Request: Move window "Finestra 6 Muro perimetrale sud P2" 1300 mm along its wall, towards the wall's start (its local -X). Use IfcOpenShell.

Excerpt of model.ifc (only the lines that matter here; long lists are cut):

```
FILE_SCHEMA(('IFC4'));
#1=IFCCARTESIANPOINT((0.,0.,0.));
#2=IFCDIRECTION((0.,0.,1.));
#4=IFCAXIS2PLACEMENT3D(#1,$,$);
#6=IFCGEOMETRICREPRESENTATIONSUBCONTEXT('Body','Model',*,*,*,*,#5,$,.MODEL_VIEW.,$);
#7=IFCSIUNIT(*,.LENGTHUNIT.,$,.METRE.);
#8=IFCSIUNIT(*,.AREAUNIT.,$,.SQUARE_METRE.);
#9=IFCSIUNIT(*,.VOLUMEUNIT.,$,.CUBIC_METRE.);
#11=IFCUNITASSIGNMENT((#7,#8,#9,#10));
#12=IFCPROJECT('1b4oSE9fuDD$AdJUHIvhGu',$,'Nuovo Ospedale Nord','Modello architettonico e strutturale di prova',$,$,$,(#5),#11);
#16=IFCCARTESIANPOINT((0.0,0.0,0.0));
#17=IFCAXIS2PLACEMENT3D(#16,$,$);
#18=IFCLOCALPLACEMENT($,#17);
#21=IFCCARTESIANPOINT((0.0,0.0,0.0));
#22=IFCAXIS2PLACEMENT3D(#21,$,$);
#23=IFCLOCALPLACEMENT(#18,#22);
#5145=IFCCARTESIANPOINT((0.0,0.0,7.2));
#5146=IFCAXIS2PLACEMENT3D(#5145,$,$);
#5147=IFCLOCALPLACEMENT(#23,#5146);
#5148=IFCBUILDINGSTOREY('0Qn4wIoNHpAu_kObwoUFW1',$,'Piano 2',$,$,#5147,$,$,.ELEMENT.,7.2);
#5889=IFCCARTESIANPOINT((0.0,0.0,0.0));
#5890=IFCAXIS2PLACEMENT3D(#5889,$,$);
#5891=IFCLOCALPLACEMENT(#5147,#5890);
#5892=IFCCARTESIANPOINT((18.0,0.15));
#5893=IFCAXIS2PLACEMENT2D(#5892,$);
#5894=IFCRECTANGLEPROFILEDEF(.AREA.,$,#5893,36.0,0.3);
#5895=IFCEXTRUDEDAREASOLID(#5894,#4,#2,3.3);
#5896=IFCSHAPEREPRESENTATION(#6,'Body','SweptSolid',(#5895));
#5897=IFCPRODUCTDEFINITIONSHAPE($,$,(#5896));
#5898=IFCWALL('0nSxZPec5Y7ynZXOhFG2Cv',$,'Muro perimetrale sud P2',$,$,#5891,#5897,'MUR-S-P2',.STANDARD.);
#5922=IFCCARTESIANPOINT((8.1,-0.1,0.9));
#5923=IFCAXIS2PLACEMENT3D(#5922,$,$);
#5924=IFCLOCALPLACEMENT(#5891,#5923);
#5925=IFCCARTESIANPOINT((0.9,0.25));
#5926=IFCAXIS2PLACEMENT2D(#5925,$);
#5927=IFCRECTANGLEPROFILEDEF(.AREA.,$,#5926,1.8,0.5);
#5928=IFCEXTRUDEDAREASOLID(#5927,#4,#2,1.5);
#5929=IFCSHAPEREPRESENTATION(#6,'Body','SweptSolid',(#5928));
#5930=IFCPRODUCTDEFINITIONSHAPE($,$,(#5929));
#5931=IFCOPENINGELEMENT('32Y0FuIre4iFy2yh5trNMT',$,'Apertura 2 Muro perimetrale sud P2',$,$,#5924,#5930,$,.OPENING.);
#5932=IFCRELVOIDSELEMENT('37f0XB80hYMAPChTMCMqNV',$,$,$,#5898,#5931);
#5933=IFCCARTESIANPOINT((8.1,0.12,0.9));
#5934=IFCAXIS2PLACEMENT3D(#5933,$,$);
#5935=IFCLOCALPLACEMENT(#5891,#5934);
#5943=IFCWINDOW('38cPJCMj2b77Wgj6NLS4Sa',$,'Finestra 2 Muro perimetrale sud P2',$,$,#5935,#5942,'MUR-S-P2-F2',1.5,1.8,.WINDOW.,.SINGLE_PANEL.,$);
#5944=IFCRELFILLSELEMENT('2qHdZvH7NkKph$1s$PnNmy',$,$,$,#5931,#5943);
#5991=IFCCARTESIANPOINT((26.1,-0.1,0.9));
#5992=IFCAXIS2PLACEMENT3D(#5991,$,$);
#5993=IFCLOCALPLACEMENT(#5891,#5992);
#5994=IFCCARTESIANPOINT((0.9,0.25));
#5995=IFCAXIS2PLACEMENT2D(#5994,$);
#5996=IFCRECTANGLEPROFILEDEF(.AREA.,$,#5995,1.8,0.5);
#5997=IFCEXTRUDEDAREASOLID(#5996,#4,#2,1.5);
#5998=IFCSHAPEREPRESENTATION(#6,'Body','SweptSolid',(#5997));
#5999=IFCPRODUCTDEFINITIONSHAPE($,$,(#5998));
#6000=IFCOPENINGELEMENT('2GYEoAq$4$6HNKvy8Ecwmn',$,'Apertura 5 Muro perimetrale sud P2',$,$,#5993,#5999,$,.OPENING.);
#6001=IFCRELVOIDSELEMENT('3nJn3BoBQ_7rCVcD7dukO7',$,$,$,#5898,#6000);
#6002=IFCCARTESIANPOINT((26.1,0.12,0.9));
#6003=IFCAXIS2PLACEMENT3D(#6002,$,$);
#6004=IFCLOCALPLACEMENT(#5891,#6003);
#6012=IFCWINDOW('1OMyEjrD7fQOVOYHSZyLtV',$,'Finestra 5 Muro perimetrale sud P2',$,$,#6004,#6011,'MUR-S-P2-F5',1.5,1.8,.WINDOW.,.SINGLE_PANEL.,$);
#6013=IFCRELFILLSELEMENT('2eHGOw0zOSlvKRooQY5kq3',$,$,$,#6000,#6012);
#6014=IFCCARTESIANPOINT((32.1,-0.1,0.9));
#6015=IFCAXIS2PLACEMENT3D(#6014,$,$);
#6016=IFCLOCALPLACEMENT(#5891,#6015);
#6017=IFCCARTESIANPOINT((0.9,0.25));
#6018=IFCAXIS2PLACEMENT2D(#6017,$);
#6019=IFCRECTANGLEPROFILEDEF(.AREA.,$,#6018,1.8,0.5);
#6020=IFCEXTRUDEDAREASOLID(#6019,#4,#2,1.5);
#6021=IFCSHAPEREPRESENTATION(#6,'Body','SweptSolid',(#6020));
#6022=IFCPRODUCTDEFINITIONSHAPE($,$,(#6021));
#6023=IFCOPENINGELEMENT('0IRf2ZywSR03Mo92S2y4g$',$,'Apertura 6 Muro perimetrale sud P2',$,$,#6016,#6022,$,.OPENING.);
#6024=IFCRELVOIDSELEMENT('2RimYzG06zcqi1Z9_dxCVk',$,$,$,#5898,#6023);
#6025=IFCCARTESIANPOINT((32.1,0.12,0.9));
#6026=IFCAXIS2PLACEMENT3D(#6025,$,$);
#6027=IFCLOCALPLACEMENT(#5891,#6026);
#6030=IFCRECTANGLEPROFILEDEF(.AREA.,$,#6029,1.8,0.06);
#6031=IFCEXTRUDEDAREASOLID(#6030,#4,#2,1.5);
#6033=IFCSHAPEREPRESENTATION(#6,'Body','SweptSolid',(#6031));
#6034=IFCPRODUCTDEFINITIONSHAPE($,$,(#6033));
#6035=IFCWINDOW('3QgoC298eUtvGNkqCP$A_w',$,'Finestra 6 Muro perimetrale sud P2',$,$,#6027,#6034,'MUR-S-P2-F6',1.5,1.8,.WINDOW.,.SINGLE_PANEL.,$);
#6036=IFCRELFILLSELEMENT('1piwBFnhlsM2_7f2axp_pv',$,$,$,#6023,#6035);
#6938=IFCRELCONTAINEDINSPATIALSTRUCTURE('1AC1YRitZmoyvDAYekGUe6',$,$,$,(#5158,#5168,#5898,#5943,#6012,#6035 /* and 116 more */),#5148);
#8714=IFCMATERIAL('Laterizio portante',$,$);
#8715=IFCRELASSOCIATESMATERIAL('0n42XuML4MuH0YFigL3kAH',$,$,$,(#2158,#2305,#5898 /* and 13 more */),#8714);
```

```python
import ifcopenshell
import ifcopenshell.api.geometry
import ifcopenshell.util.placement
import ifcopenshell.util.unit

model = ifcopenshell.open("model.ifc")
unit_scale = ifcopenshell.util.unit.calculate_unit_scale(model)

window = model.by_guid("3QgoC298eUtvGNkqCP$A_w")
opening = window.FillsVoids[0].RelatingOpeningElement
wall = opening.VoidsElements[0].RelatingBuildingElement

wall_matrix = ifcopenshell.util.placement.get_local_placement(wall.ObjectPlacement)
shift = wall_matrix[:3, 0] * -1.3 / unit_scale
before = ifcopenshell.util.placement.get_local_placement(window.ObjectPlacement)[:3, 3].copy()

# The window is not placed relative to its opening, so move both.
for product in (opening, window):
    matrix = ifcopenshell.util.placement.get_local_placement(product.ObjectPlacement)
    matrix[:3, 3] += shift
    ifcopenshell.api.geometry.edit_object_placement(model, product=product, matrix=matrix, is_si=False)

after = ifcopenshell.util.placement.get_local_placement(window.ObjectPlacement)[:3, 3]
print("window moved by", (after - before).round(3) + 0.0)

model.write("model_edited.ifc")
```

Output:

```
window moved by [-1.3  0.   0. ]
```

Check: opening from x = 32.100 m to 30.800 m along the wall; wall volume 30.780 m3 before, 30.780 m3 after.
